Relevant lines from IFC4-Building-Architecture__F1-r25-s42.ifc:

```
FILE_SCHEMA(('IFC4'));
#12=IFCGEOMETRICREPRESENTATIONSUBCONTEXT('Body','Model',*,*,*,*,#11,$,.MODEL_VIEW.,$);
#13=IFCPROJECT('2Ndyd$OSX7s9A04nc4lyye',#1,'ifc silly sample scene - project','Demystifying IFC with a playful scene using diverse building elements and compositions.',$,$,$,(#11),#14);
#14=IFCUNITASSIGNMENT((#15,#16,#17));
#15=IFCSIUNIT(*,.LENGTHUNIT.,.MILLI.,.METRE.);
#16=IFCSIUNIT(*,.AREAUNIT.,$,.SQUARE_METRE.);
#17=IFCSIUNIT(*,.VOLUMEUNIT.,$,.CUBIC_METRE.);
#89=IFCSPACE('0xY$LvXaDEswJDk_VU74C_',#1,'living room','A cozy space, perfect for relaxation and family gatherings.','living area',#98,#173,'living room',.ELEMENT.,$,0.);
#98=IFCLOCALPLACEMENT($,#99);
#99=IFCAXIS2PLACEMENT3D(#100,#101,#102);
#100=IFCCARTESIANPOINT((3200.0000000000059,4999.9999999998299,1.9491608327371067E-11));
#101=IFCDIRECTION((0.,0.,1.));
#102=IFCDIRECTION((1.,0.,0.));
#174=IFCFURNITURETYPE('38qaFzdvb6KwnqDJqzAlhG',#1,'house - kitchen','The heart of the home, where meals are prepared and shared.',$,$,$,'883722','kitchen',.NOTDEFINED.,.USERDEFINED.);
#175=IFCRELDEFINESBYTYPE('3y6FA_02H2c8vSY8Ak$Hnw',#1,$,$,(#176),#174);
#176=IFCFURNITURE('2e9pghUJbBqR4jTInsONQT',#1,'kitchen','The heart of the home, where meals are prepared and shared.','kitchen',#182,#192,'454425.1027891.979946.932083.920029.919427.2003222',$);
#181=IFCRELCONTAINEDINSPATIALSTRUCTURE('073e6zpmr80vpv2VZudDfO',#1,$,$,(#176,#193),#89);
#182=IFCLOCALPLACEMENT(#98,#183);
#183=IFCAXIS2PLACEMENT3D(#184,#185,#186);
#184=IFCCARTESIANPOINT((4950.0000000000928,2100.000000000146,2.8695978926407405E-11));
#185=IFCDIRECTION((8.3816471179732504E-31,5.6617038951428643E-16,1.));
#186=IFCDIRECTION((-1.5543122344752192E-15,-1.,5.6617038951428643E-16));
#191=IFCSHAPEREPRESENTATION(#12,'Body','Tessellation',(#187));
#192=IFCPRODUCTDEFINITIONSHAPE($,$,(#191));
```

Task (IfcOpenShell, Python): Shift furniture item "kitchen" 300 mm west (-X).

```python
import ifcopenshell
import ifcopenshell.api.geometry
import ifcopenshell.util.placement
import ifcopenshell.util.unit

model = ifcopenshell.open("IFC4-Building-Architecture__F1-r25-s42.ifc")
unit_scale = ifcopenshell.util.unit.calculate_unit_scale(model)

item = model.by_guid("2e9pghUJbBqR4jTInsONQT")
matrix = ifcopenshell.util.placement.get_local_placement(item.ObjectPlacement)
matrix[0, 3] -= 0.3 / unit_scale
ifcopenshell.api.geometry.edit_object_placement(model, product=item, matrix=matrix, is_si=False)

print(ifcopenshell.util.placement.get_local_placement(item.ObjectPlacement).round(3) + 0.0)

model.write("IFC4-Building-Architecture__F1-r25-s42_edited.ifc")
```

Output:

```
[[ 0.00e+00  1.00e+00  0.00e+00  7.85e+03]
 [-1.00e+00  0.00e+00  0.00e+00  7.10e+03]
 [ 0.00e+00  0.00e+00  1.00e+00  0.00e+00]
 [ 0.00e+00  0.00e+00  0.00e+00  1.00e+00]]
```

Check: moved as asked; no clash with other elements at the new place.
